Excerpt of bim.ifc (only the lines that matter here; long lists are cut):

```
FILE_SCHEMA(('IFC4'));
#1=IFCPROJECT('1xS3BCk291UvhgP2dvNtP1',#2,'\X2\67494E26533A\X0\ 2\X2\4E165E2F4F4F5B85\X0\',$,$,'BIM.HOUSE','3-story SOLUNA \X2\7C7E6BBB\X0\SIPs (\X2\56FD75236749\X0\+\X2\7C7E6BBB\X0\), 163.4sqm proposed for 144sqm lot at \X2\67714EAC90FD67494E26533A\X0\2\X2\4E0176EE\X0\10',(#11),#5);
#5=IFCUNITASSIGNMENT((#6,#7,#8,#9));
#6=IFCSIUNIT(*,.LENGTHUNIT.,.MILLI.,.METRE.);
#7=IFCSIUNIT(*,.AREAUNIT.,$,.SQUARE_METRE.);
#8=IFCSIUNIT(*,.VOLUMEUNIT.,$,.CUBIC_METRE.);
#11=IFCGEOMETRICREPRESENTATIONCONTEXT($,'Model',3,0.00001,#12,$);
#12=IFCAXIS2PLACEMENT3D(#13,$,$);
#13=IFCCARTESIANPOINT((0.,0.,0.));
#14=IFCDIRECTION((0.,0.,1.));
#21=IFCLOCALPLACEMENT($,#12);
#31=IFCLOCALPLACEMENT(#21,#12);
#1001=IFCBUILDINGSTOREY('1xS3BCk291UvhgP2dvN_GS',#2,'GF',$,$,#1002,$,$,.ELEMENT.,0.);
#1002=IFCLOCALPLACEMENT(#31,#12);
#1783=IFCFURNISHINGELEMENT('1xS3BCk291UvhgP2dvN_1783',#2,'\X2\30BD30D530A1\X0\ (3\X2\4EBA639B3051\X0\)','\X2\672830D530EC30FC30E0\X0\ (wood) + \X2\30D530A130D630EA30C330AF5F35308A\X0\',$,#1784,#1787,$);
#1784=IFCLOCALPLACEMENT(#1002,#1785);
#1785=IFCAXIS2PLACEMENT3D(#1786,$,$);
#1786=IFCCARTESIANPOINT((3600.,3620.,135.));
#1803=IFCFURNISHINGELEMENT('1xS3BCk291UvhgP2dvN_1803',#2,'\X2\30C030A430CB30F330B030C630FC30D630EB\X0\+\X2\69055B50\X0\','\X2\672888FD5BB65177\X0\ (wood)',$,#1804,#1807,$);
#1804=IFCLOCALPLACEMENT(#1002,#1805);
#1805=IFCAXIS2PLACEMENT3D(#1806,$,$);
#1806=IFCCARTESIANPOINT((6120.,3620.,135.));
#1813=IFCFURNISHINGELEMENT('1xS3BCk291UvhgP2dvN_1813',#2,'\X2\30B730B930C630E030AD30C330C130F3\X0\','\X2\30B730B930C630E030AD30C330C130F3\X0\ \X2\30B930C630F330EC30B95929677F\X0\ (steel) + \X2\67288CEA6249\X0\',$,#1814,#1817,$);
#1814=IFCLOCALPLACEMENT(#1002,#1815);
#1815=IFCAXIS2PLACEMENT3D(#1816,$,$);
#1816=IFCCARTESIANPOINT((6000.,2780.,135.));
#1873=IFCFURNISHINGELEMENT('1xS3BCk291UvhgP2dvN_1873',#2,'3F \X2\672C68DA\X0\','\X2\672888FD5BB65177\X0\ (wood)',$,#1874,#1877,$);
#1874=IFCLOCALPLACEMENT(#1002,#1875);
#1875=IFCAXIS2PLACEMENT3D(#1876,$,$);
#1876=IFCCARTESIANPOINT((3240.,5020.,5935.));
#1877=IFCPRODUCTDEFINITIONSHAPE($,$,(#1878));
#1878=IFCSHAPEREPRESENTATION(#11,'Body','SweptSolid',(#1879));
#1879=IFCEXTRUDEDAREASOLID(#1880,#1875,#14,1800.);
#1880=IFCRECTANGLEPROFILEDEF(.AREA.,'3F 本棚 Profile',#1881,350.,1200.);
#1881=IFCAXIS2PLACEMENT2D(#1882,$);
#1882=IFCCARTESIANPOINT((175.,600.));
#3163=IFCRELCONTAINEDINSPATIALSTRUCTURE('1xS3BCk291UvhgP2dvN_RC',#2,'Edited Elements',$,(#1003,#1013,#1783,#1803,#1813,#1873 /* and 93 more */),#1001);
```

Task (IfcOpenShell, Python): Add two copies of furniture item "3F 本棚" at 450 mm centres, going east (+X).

```python
import numpy as np
import ifcopenshell
import ifcopenshell.api.geometry
import ifcopenshell.api.root
import ifcopenshell.util.element
import ifcopenshell.util.placement
import ifcopenshell.util.unit

model = ifcopenshell.open("bim.ifc")
unit_scale = ifcopenshell.util.unit.calculate_unit_scale(model)


def reuse_history(source, copy):
    """copy_class also copies each property set's owner history, people and application; keep the originals."""
    for rel in copy.IsDefinedBy:
        if rel.is_a("IfcRelDefinesByProperties") and (history := rel.RelatingPropertyDefinition.OwnerHistory):
            rel.RelatingPropertyDefinition.OwnerHistory = source.OwnerHistory
            ifcopenshell.util.element.remove_deep2(model, history)


source = model.by_id(1873)
base = ifcopenshell.util.placement.get_local_placement(source.ObjectPlacement)
step = np.array([1.0, 0.0, 0.0]) * 0.45 / unit_scale

for i in range(1, 3):
    copy = ifcopenshell.api.root.copy_class(model, product=source)
    copy.Representation = ifcopenshell.util.element.copy_deep(
        model, source.Representation, exclude=["IfcGeometricRepresentationContext", "IfcRepresentationMap"]
    )
    reuse_history(source, copy)
    matrix = base.copy()
    matrix[:3, 3] += i * step
    print("added at", matrix[:3, 3].round(3) + 0.0)
    ifcopenshell.api.geometry.edit_object_placement(model, product=copy, matrix=matrix, is_si=False)

model.write("bim-out.ifc")
```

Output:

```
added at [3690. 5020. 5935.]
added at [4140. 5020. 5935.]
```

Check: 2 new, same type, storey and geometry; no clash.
